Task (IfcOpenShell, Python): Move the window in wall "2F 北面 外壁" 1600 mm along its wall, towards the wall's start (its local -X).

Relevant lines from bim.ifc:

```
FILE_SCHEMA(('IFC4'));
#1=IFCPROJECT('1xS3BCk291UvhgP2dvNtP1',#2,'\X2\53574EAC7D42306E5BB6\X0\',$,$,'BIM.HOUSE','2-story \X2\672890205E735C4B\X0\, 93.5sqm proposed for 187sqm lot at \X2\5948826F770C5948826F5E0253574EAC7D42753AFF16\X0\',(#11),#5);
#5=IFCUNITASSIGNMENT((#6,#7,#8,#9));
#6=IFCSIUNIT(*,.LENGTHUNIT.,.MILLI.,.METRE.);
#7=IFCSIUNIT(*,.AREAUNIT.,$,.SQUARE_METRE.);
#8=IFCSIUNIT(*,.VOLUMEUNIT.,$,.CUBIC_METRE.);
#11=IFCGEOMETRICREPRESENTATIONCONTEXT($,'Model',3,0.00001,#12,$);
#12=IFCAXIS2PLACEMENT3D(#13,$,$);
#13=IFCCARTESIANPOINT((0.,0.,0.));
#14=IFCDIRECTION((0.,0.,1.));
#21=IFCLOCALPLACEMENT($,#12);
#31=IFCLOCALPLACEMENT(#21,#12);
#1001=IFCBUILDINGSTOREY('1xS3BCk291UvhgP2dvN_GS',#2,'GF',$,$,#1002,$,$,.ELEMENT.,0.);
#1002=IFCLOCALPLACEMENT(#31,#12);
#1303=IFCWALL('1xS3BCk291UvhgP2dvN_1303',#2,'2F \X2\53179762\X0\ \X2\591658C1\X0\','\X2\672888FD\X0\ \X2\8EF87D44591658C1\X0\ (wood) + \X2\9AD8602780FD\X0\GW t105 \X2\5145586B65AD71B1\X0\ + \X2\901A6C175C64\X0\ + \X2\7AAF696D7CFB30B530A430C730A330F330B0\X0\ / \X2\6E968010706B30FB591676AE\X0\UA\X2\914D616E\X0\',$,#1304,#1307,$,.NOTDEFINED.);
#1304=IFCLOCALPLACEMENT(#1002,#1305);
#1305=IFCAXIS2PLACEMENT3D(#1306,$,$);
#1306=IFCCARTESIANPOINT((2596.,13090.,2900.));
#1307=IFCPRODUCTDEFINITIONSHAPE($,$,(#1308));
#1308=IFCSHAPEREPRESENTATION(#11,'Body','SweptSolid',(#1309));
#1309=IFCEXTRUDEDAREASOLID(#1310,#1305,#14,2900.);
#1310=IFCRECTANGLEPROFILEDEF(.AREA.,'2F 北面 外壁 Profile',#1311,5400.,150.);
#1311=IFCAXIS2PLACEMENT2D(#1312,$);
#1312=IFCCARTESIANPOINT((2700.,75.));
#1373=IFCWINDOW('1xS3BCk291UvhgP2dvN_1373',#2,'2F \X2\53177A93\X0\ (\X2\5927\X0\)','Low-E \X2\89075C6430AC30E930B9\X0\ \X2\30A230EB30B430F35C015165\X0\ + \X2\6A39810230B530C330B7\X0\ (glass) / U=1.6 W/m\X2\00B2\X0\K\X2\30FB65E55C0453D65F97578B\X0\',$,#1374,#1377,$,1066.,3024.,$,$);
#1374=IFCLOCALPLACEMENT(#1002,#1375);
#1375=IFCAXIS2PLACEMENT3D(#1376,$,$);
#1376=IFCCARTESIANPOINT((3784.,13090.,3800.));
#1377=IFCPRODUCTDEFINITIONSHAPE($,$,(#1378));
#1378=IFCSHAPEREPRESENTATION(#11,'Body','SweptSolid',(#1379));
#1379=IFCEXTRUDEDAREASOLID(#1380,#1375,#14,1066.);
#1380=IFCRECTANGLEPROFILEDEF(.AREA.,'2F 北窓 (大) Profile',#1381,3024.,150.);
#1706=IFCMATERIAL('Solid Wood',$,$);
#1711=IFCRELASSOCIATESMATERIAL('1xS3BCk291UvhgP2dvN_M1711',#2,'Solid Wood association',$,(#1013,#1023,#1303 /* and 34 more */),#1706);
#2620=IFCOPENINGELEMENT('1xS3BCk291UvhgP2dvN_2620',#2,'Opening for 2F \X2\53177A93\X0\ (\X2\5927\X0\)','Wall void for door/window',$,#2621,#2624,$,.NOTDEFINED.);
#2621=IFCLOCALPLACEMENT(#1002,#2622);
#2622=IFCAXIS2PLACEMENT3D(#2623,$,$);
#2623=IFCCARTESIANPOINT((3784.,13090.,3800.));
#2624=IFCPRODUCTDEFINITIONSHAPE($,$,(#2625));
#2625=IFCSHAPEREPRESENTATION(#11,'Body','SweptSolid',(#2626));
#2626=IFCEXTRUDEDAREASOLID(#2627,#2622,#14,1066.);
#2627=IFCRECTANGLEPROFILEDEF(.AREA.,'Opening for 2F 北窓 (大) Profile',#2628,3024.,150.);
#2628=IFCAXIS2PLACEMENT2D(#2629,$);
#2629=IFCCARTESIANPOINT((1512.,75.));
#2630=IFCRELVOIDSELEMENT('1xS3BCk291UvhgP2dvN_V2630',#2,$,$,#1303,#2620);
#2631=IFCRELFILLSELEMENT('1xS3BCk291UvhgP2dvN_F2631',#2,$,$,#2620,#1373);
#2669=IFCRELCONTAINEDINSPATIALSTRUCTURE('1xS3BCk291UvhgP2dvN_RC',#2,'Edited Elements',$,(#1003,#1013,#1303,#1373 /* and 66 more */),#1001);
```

```python
import ifcopenshell
import ifcopenshell.api.geometry
import ifcopenshell.util.placement
import ifcopenshell.util.unit

model = ifcopenshell.open("bim.ifc")
unit_scale = ifcopenshell.util.unit.calculate_unit_scale(model)

window = model.by_guid("1xS3BCk291UvhgP2dvN_1373")
opening = window.FillsVoids[0].RelatingOpeningElement
wall = opening.VoidsElements[0].RelatingBuildingElement

wall_matrix = ifcopenshell.util.placement.get_local_placement(wall.ObjectPlacement)
shift = wall_matrix[:3, 0] * -1.6 / unit_scale
before = ifcopenshell.util.placement.get_local_placement(window.ObjectPlacement)[:3, 3].copy()

# The window is not placed relative to its opening, so move both.
for product in (opening, window):
    matrix = ifcopenshell.util.placement.get_local_placement(product.ObjectPlacement)
    matrix[:3, 3] += shift
    ifcopenshell.api.geometry.edit_object_placement(model, product=product, matrix=matrix, is_si=False)

after = ifcopenshell.util.placement.get_local_placement(window.ObjectPlacement)[:3, 3]
print("window moved by", (after - before).round(3) + 0.0)

model.write("bim_edited.ifc")
```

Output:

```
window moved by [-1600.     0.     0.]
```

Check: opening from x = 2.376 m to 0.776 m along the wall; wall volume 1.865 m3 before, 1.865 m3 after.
